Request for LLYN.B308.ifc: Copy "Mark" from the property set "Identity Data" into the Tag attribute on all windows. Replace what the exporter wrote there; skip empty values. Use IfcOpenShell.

First a look at what the model holds.

```python
import ifcopenshell
import ifcopenshell.util.element

model = ifcopenshell.open("LLYN.B308.ifc")
print(model.schema)
windows = model.by_type("IfcWindow")
print(len(windows), "windows")
for e in windows[:8]:
    source = ifcopenshell.util.element.get_pset(e, "Identity Data", "Mark")
    target = e.Tag
    print(e.id(), repr(source), repr(target), sep=" | ")
```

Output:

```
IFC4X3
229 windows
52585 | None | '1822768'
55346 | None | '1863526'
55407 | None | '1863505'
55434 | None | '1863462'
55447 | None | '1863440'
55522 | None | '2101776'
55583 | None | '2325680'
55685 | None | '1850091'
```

```python
import ifcopenshell
import ifcopenshell.util.element

model = ifcopenshell.open("LLYN.B308.ifc")

count = 0
for e in model.by_type("IfcWindow"):
    value = ifcopenshell.util.element.get_pset(e, "Identity Data", "Mark")
    current = e.Tag
    if not value or not value.strip() or current == value:
        continue
    e.Tag = value
    count += 1

print(count, "windows updated")

model.write("LLYN.B308_rev.ifc")
```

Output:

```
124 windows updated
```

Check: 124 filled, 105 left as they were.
